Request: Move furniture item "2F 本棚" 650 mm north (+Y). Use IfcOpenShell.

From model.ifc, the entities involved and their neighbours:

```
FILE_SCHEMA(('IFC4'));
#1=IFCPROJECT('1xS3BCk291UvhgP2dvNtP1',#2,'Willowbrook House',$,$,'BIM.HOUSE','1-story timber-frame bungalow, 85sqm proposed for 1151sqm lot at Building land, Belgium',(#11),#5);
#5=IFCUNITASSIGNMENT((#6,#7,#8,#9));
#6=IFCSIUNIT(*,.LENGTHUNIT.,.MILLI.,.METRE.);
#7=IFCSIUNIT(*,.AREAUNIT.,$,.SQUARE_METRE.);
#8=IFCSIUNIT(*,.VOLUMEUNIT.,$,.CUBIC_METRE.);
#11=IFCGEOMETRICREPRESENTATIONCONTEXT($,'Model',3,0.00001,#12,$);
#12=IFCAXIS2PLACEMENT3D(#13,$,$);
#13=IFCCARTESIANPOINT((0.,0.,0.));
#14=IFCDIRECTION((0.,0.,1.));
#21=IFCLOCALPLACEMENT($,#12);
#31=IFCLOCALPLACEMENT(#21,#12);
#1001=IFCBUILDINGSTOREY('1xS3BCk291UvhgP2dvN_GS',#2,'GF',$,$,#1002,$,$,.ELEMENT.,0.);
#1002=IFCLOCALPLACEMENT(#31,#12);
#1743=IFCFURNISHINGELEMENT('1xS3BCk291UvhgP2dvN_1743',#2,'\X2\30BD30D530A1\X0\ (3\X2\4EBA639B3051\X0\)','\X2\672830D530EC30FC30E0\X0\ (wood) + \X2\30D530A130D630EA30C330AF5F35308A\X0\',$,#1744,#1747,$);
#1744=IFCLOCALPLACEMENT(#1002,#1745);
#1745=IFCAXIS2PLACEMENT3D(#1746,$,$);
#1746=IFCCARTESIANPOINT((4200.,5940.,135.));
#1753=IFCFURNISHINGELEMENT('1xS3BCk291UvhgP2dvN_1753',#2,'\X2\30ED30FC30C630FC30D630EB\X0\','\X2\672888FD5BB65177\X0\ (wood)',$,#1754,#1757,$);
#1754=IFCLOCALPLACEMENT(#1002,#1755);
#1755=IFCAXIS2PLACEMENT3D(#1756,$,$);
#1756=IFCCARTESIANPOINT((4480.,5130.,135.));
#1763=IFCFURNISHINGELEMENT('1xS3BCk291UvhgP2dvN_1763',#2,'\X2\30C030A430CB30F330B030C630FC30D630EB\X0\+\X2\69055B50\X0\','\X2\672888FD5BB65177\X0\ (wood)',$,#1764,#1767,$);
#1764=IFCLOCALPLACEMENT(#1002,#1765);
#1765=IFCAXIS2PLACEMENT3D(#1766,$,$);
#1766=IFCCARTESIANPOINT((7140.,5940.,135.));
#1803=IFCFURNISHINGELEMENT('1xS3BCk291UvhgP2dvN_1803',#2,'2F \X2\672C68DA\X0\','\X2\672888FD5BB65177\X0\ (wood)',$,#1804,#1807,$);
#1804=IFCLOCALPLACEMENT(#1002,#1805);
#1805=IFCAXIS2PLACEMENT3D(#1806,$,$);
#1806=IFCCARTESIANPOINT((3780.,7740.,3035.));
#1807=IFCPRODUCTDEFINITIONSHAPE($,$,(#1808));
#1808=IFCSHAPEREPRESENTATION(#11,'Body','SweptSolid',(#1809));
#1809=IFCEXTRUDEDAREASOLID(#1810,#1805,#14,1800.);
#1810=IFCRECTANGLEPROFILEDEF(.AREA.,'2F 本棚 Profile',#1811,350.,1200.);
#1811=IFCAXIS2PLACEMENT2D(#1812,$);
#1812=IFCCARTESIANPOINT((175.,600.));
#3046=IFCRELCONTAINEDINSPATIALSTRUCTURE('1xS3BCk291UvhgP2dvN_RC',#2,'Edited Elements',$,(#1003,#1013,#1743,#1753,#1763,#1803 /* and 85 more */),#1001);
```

```python
import ifcopenshell
import ifcopenshell.api.geometry
import ifcopenshell.util.placement

model = ifcopenshell.open("model.ifc")

item = model.by_id(1803)
matrix = ifcopenshell.util.placement.get_local_placement(item.ObjectPlacement)
matrix[1, 3] += 650.0
ifcopenshell.api.geometry.edit_object_placement(model, product=item, matrix=matrix, is_si=False)

print(ifcopenshell.util.placement.get_local_placement(item.ObjectPlacement).round(3) + 0.0)

model.write("model_v2.ifc")
```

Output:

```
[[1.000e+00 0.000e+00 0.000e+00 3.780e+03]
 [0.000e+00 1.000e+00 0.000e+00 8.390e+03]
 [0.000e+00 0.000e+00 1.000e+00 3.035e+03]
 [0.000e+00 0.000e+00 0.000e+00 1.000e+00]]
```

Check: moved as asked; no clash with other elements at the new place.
